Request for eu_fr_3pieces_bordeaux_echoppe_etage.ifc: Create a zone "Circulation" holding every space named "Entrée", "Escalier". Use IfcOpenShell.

First a look at what the model holds.

```python
import ifcopenshell

model = ifcopenshell.open("eu_fr_3pieces_bordeaux_echoppe_etage.ifc")
print(model.schema)
seen = {}
for space in model.by_type("IfcSpace"):
    seen[space.LongName] = seen.get(space.LongName, 0) + 1
for name, count in sorted(seen.items(), key=str):
    print(count, "x", name)
print("zones:", [z.Name for z in model.by_type("IfcZone")][:20])
```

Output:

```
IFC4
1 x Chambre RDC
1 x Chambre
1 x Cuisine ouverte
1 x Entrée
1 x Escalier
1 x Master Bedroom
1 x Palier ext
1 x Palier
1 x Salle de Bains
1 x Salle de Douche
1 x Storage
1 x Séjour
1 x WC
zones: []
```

```python
import ifcopenshell
import ifcopenshell.api.group
import ifcopenshell.api.root

model = ifcopenshell.open("eu_fr_3pieces_bordeaux_echoppe_etage.ifc")

names = {"Entrée", "Escalier"}
spaces = [s for s in model.by_type("IfcSpace") if s.LongName in names]

zone = ifcopenshell.api.root.create_entity(model, ifc_class="IfcZone", name="Circulation")
ifcopenshell.api.group.assign_group(model, products=spaces, group=zone)
print(len(spaces), "spaces in", zone.Name)

model.write("eu_fr_3pieces_bordeaux_echoppe_etage_v2.ifc")
```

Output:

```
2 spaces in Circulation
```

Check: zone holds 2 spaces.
